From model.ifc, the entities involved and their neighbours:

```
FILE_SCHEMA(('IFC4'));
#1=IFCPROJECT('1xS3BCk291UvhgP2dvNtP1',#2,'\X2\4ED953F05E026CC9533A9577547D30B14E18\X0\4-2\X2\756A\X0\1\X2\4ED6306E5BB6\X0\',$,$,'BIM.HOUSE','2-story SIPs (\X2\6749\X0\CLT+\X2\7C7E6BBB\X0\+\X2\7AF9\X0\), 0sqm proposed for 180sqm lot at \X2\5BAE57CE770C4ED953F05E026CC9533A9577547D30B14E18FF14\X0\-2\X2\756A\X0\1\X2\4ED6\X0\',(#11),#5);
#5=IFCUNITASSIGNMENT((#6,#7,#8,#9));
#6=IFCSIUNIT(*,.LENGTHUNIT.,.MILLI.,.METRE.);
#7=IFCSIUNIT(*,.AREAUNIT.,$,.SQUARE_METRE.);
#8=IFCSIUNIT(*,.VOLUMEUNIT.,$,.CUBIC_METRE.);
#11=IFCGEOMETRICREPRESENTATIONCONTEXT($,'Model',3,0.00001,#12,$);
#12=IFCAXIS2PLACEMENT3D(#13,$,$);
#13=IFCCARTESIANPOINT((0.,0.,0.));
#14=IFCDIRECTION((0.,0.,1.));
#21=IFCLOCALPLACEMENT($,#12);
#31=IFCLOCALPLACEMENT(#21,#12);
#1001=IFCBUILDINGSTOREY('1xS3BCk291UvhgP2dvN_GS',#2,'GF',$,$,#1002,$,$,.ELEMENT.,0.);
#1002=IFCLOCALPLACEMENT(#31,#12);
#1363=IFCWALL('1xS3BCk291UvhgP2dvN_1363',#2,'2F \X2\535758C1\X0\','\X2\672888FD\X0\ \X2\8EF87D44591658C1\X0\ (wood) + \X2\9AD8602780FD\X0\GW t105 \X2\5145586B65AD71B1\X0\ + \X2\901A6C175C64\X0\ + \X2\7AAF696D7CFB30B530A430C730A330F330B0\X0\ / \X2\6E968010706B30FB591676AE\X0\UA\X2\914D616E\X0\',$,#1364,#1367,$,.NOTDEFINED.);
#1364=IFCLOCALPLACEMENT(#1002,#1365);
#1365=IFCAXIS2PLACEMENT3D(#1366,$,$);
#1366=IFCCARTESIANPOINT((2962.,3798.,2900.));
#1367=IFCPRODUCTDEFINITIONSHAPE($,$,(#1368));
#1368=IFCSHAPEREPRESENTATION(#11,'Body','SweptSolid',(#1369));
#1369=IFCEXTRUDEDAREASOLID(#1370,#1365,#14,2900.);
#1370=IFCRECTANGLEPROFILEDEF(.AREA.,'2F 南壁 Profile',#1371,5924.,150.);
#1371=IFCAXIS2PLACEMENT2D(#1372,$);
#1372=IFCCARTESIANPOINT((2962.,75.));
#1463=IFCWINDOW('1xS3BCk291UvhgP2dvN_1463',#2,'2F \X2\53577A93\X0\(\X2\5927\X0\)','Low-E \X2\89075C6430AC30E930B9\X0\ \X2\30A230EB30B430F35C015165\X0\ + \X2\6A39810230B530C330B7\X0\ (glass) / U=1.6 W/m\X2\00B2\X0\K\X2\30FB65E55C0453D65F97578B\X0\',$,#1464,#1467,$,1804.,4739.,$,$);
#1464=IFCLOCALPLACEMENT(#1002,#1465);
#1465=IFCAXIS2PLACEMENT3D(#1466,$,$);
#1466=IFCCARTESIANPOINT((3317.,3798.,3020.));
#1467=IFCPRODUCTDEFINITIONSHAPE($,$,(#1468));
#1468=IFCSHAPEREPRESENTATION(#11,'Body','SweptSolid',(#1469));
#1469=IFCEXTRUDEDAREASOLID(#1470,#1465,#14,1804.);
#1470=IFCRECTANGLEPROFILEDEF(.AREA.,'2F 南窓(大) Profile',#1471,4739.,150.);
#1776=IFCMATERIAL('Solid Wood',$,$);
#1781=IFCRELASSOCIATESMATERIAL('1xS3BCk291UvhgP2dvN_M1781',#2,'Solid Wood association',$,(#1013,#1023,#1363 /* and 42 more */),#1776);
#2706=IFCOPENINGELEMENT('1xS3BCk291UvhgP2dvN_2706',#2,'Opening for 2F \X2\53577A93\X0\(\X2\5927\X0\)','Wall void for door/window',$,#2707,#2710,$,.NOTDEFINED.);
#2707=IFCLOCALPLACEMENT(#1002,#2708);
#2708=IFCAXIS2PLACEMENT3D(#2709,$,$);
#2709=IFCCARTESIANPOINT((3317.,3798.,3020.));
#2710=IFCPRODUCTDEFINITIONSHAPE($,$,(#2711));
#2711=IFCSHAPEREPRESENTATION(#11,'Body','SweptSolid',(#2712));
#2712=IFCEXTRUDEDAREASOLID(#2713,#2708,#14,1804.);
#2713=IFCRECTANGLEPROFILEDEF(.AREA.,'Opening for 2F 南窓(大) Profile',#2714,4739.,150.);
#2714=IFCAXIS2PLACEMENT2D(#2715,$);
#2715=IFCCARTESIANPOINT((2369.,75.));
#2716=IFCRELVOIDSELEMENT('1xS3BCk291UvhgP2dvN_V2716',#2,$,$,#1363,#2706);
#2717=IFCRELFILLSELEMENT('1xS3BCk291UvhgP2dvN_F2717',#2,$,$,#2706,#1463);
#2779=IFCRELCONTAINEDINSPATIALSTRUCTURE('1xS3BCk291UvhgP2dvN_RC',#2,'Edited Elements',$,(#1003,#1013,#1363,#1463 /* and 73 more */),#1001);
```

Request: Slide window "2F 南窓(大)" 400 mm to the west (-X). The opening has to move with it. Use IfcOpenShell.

```python
import ifcopenshell
import ifcopenshell.api.geometry
import ifcopenshell.util.placement
import ifcopenshell.util.unit

model = ifcopenshell.open("model.ifc")
unit_scale = ifcopenshell.util.unit.calculate_unit_scale(model)

window = model.by_id(1463)
opening = window.FillsVoids[0].RelatingOpeningElement
wall = opening.VoidsElements[0].RelatingBuildingElement

wall_matrix = ifcopenshell.util.placement.get_local_placement(wall.ObjectPlacement)
shift = wall_matrix[:3, 0] * -0.4 / unit_scale
before = ifcopenshell.util.placement.get_local_placement(window.ObjectPlacement)[:3, 3].copy()

# The window is not placed relative to its opening, so move both.
for product in (opening, window):
    matrix = ifcopenshell.util.placement.get_local_placement(product.ObjectPlacement)
    matrix[:3, 3] += shift
    ifcopenshell.api.geometry.edit_object_placement(model, product=product, matrix=matrix, is_si=False)

after = ifcopenshell.util.placement.get_local_placement(window.ObjectPlacement)[:3, 3]
print("window moved by", (after - before).round(3) + 0.0)

model.write("model_edited.ifc")
```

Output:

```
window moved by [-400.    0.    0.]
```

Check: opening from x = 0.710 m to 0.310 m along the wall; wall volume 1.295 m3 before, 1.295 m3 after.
